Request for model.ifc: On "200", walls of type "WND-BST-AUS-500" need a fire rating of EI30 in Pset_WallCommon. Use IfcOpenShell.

First a look at what the model holds.

```python
import ifcopenshell
import ifcopenshell.util.element

model = ifcopenshell.open("model.ifc")
print(model.schema)
storey = next(s for s in model.by_type("IfcBuildingStorey") if s.Name == "200")
walls = [e for e in ifcopenshell.util.element.get_decomposition(storey) if e.is_a("IfcWall")]
seen = {}
for e in walls:
    element_type = ifcopenshell.util.element.get_type(e)
    key = (element_type.Name if element_type != e and element_type else None, ifcopenshell.util.element.get_pset(e, "Pset_WallCommon", "FireRating"))
    seen[key] = seen.get(key, 0) + 1
for (name, value), count in sorted(seen.items(), key=str):
    print(count, "x", name, "|", value)
```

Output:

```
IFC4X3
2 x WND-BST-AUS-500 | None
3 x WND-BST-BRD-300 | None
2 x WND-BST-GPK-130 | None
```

```python
import ifcopenshell
import ifcopenshell.api.pset
import ifcopenshell.util.element

model = ifcopenshell.open("model.ifc")

storey = next(s for s in model.by_type("IfcBuildingStorey") if s.Name == "200")
walls = [e for e in ifcopenshell.util.element.get_decomposition(storey) if e.is_a("IfcWall")]

count = 0
for e in walls:
    element_type = ifcopenshell.util.element.get_type(e)
    if element_type in (None, e) or element_type.Name != "WND-BST-AUS-500":
        continue
    # add_pset returns the element's existing set when there is one.
    pset = ifcopenshell.api.pset.add_pset(model, product=e, name="Pset_WallCommon")
    ifcopenshell.api.pset.edit_pset(model, pset=pset, properties={"FireRating": "EI30"})
    count += 1

print(count, "walls updated")

model.write("model_v2.ifc")
```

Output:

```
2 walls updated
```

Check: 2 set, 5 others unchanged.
